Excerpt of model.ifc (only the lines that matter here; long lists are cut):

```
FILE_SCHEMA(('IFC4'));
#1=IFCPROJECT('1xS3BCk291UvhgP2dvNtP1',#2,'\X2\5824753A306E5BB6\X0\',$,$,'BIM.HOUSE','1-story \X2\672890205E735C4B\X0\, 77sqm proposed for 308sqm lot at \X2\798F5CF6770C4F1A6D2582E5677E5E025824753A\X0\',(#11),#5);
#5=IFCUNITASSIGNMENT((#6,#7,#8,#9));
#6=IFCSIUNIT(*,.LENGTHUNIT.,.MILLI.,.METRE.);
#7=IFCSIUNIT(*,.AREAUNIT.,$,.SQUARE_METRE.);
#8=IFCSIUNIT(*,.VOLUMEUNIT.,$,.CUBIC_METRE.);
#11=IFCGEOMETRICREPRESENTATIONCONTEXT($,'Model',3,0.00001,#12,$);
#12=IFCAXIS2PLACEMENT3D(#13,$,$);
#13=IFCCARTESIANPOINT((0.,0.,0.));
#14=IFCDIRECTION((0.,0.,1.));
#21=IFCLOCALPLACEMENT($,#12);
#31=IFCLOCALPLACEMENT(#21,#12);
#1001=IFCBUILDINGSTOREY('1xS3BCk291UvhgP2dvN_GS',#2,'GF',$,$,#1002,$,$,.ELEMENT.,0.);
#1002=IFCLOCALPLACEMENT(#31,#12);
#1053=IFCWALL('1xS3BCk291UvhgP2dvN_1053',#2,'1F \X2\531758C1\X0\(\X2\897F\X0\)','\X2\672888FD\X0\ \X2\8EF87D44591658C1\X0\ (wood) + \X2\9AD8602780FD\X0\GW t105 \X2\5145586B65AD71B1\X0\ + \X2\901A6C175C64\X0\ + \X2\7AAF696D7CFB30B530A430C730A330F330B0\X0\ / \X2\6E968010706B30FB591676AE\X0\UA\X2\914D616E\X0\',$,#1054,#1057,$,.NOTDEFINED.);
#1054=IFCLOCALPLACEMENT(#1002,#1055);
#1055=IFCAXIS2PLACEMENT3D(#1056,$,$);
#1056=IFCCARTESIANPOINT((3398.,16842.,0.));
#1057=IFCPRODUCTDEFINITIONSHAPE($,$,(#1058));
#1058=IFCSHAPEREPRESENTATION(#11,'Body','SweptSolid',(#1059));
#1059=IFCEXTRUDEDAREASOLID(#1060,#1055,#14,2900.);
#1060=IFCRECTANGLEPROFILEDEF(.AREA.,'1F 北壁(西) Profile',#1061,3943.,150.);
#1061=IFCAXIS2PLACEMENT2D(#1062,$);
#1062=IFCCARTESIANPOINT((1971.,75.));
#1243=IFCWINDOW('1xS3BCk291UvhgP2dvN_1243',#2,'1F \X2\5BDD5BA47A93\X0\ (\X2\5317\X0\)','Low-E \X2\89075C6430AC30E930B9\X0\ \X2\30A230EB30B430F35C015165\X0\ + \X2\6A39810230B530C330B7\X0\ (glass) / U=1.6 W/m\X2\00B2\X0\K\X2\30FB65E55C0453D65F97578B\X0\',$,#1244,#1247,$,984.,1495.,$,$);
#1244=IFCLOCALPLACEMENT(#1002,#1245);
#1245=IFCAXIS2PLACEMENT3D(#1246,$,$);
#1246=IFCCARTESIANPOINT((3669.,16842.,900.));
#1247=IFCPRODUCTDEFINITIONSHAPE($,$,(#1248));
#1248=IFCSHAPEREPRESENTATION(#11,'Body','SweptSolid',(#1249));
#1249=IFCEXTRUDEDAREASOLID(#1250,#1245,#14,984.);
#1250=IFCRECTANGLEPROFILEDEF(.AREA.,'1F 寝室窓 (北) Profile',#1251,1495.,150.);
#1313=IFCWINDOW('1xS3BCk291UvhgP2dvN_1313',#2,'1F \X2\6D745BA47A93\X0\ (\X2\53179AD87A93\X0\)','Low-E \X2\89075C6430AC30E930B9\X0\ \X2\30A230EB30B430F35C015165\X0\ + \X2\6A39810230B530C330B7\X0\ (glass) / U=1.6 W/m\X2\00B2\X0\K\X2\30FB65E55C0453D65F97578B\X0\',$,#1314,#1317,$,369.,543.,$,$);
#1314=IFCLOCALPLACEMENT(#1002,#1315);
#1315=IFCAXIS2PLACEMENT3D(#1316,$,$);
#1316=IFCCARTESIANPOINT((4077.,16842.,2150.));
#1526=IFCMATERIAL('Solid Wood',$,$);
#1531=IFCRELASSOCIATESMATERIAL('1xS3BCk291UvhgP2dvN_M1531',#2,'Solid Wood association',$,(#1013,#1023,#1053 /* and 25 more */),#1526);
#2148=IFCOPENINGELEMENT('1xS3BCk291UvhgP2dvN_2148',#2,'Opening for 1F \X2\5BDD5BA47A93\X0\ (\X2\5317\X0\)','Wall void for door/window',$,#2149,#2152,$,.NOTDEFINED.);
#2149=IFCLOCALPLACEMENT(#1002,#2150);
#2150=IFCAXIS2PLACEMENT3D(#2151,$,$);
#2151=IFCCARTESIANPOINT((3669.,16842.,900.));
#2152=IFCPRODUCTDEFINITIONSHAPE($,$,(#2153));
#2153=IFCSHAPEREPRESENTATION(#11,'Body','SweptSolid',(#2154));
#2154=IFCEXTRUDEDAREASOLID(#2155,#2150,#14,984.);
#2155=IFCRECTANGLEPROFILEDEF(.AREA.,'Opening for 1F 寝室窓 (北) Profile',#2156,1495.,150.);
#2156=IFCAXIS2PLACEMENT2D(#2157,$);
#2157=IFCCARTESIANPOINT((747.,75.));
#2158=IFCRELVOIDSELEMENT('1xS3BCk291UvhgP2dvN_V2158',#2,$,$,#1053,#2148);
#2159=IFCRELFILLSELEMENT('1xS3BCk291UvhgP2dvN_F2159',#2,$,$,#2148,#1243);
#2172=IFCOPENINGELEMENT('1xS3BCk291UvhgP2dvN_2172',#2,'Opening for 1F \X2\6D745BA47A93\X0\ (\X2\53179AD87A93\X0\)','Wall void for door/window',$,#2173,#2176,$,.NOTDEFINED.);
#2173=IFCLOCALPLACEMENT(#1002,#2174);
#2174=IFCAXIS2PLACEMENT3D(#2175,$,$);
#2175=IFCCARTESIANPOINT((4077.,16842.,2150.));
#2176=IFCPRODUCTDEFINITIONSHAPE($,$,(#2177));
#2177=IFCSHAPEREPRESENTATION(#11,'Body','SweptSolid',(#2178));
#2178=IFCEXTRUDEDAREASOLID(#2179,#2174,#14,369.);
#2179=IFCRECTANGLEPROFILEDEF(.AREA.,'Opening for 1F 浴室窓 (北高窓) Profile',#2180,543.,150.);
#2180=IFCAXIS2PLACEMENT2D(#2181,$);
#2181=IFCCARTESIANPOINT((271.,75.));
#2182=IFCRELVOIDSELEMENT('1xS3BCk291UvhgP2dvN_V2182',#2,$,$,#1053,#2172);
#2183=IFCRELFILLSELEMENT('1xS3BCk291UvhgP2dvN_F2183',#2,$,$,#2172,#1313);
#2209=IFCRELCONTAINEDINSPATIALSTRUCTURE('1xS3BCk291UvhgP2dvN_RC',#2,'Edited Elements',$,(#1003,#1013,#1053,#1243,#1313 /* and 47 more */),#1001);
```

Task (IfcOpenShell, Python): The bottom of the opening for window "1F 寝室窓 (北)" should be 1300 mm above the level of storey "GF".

```python
import numpy as np
import ifcopenshell
import ifcopenshell.api.geometry
import ifcopenshell.geom
import ifcopenshell.util.element
import ifcopenshell.util.placement
import ifcopenshell.util.shape
import ifcopenshell.util.unit

model = ifcopenshell.open("model.ifc")
unit_scale = ifcopenshell.util.unit.calculate_unit_scale(model)

window = model.by_guid("1xS3BCk291UvhgP2dvN_1243")
opening = window.FillsVoids[0].RelatingOpeningElement
storey = ifcopenshell.util.element.get_container(window, ifc_class="IfcBuildingStorey")
level = ifcopenshell.util.placement.get_local_placement(storey.ObjectPlacement)[2, 3]

# The opening's origin need not be at the sill, so measure its lowest point.
shape = ifcopenshell.geom.create_shape(ifcopenshell.geom.settings(), opening)
bottom = ifcopenshell.util.shape.get_shape_bottom_elevation(shape, shape.geometry) / unit_scale
dz = level + 1.3 / unit_scale - bottom

shift = np.array([0.0, 0.0, dz])
# The window is not placed relative to its opening, so move both.
for product in (opening, window):
    matrix = ifcopenshell.util.placement.get_local_placement(product.ObjectPlacement)
    matrix[:3, 3] += shift
    ifcopenshell.api.geometry.edit_object_placement(model, product=product, matrix=matrix, is_si=False)

print(f"moved by {dz * unit_scale:+.3f} m")

model.write("model_v2.ifc")
```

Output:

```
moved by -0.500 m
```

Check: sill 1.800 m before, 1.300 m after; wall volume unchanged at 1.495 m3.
